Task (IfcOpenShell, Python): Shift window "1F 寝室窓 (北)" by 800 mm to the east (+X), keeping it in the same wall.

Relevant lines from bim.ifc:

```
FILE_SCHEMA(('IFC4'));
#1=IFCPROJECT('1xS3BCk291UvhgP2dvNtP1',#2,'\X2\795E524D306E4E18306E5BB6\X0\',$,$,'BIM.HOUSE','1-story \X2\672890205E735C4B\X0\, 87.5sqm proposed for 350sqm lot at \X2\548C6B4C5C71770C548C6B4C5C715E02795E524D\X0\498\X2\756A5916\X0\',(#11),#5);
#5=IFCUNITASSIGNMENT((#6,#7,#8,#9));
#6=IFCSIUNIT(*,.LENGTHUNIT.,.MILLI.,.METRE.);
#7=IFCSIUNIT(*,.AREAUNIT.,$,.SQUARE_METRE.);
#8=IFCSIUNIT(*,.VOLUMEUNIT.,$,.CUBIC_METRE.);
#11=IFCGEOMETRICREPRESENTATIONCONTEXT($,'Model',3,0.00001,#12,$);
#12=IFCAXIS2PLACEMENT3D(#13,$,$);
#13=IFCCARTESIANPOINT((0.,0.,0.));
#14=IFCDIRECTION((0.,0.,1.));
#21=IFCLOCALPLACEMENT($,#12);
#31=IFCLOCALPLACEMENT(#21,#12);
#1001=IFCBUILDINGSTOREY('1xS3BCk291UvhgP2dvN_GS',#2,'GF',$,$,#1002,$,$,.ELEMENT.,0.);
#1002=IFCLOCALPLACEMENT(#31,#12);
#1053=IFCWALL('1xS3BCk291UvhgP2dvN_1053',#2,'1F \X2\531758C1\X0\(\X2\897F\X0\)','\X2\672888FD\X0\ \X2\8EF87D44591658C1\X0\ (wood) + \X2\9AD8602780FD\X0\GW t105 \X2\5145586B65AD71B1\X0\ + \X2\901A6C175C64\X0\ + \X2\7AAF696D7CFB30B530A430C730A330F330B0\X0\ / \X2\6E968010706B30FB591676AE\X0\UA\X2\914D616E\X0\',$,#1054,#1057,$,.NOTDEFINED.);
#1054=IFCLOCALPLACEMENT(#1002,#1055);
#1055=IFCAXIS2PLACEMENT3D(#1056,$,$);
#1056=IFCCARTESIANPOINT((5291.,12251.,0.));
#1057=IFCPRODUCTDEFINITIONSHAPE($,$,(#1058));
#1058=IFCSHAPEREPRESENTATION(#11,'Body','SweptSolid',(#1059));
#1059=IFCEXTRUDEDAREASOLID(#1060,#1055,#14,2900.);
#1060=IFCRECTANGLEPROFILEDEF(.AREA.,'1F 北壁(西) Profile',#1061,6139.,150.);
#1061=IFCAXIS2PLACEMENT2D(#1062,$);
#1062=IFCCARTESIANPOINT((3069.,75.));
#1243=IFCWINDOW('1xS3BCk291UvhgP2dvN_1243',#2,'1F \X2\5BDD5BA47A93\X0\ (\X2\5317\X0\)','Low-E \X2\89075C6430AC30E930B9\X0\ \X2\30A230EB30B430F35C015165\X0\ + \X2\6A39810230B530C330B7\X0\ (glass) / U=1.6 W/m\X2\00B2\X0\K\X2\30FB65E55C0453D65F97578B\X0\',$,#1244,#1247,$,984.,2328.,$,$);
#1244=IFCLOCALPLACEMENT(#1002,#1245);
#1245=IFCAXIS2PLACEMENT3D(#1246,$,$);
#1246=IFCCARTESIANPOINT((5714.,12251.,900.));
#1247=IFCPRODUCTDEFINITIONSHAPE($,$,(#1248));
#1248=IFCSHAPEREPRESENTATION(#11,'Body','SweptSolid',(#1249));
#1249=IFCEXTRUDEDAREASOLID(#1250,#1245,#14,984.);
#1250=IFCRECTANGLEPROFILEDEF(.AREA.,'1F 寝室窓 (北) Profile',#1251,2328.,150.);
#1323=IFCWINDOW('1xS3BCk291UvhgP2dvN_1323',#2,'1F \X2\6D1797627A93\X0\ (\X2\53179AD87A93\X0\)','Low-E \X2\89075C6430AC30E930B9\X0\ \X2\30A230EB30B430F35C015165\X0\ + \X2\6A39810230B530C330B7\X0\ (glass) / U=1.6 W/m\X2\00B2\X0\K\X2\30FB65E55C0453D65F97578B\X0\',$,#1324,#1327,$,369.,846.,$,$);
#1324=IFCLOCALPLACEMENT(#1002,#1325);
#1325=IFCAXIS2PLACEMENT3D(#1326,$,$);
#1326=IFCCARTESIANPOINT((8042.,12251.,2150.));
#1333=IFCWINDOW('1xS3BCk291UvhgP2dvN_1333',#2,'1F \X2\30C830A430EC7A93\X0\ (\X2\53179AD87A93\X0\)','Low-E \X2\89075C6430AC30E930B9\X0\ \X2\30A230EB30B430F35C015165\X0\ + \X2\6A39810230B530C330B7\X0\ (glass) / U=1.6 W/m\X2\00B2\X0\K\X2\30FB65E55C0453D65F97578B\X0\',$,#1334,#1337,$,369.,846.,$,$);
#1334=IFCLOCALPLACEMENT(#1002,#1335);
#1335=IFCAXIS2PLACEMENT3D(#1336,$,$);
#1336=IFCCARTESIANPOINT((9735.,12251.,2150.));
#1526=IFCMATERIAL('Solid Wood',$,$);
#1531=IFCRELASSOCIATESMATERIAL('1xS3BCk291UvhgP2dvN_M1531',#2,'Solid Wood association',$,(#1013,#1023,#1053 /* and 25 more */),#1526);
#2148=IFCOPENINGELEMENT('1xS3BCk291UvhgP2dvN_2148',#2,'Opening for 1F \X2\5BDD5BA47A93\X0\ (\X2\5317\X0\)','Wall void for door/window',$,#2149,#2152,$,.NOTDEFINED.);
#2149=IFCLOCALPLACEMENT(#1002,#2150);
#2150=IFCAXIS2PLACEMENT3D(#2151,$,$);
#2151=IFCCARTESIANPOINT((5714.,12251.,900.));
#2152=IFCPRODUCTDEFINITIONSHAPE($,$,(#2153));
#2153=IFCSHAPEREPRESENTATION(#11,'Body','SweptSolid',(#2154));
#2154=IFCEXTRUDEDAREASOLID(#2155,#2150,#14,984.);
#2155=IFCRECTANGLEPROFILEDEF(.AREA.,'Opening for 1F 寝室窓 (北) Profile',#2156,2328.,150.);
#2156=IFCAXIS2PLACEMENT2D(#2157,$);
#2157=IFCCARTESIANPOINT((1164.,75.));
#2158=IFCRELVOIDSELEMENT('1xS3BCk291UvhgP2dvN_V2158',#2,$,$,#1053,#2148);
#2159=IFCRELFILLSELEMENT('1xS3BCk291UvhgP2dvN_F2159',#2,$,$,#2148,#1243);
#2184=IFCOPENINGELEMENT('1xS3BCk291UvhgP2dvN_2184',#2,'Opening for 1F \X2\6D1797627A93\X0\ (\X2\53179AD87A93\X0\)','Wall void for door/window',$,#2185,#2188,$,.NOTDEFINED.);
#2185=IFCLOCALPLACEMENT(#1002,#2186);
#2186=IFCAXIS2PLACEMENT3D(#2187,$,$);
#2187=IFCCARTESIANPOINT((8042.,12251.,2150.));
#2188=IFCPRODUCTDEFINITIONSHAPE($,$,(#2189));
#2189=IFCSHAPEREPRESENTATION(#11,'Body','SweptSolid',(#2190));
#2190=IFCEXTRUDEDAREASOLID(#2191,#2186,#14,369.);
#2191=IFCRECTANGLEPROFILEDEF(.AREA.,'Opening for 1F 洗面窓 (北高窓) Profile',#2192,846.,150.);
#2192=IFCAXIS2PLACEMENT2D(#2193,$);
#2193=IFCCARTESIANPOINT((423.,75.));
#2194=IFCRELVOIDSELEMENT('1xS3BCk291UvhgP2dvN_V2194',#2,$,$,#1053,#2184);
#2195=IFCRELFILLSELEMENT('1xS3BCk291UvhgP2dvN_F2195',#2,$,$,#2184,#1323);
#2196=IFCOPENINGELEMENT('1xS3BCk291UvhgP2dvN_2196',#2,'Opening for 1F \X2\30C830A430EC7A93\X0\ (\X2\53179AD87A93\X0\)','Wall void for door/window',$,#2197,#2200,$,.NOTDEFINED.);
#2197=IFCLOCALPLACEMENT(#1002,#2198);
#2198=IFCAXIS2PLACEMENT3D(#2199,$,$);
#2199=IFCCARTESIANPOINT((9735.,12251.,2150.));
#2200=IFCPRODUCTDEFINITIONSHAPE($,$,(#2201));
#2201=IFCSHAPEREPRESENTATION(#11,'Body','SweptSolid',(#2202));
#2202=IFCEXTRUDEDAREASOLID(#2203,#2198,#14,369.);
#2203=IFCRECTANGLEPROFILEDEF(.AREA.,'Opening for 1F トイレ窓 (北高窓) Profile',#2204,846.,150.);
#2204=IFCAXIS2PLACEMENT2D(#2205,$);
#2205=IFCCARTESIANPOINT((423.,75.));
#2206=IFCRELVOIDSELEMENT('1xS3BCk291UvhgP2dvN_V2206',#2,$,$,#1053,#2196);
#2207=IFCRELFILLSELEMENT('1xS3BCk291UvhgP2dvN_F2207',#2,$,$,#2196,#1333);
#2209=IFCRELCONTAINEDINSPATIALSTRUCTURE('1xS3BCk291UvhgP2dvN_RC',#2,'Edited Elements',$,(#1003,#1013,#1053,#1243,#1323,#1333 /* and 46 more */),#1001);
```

```python
import ifcopenshell
import ifcopenshell.api.geometry
import ifcopenshell.util.placement

model = ifcopenshell.open("bim.ifc")

window = model.by_guid("1xS3BCk291UvhgP2dvN_1243")
opening = window.FillsVoids[0].RelatingOpeningElement
wall = opening.VoidsElements[0].RelatingBuildingElement

wall_matrix = ifcopenshell.util.placement.get_local_placement(wall.ObjectPlacement)
shift = wall_matrix[:3, 0] * 800.0
before = ifcopenshell.util.placement.get_local_placement(window.ObjectPlacement)[:3, 3].copy()

# The window is not placed relative to its opening, so move both.
for product in (opening, window):
    matrix = ifcopenshell.util.placement.get_local_placement(product.ObjectPlacement)
    matrix[:3, 3] += shift
    ifcopenshell.api.geometry.edit_object_placement(model, product=product, matrix=matrix, is_si=False)

after = ifcopenshell.util.placement.get_local_placement(window.ObjectPlacement)[:3, 3]
print("window moved by", (after - before).round(3) + 0.0)

model.write("bim_edited.ifc")
```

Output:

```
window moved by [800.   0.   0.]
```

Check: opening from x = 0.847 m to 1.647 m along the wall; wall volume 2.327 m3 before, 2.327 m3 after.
